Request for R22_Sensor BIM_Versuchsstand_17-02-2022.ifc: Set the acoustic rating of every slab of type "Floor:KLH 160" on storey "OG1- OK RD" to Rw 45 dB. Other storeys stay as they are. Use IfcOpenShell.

First a look at what the model holds.

```python
import ifcopenshell
import ifcopenshell.util.element

model = ifcopenshell.open("R22_Sensor BIM_Versuchsstand_17-02-2022.ifc")
print(model.schema)
storey = next(s for s in model.by_type("IfcBuildingStorey") if s.Name == "OG1- OK RD")
slabs = [e for e in ifcopenshell.util.element.get_decomposition(storey) if e.is_a("IfcSlab")]
seen = {}
for e in slabs:
    element_type = ifcopenshell.util.element.get_type(e)
    key = (element_type.Name if element_type != e and element_type else None, ifcopenshell.util.element.get_pset(e, "Pset_SlabCommon", "AcousticRating"))
    seen[key] = seen.get(key, 0) + 1
for (name, value), count in sorted(seen.items(), key=str):
    print(count, "x", name, "|", value)
```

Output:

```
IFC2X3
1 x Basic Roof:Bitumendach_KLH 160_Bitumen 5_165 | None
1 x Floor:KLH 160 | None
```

```python
import ifcopenshell
import ifcopenshell.api.pset
import ifcopenshell.util.element

model = ifcopenshell.open("R22_Sensor BIM_Versuchsstand_17-02-2022.ifc")

storey = next(s for s in model.by_type("IfcBuildingStorey") if s.Name == "OG1- OK RD")
slabs = [e for e in ifcopenshell.util.element.get_decomposition(storey) if e.is_a("IfcSlab")]

count = 0
for e in slabs:
    element_type = ifcopenshell.util.element.get_type(e)
    if element_type in (None, e) or element_type.Name != "Floor:KLH 160":
        continue
    # add_pset returns the element's existing set when there is one.
    pset = ifcopenshell.api.pset.add_pset(model, product=e, name="Pset_SlabCommon")
    ifcopenshell.api.pset.edit_pset(model, pset=pset, properties={"AcousticRating": "Rw 45 dB"})
    count += 1

print(count, "slabs updated")

model.write("R22_Sensor BIM_Versuchsstand_17-02-2022_edited.ifc")
```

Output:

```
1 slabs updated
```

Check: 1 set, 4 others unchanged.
